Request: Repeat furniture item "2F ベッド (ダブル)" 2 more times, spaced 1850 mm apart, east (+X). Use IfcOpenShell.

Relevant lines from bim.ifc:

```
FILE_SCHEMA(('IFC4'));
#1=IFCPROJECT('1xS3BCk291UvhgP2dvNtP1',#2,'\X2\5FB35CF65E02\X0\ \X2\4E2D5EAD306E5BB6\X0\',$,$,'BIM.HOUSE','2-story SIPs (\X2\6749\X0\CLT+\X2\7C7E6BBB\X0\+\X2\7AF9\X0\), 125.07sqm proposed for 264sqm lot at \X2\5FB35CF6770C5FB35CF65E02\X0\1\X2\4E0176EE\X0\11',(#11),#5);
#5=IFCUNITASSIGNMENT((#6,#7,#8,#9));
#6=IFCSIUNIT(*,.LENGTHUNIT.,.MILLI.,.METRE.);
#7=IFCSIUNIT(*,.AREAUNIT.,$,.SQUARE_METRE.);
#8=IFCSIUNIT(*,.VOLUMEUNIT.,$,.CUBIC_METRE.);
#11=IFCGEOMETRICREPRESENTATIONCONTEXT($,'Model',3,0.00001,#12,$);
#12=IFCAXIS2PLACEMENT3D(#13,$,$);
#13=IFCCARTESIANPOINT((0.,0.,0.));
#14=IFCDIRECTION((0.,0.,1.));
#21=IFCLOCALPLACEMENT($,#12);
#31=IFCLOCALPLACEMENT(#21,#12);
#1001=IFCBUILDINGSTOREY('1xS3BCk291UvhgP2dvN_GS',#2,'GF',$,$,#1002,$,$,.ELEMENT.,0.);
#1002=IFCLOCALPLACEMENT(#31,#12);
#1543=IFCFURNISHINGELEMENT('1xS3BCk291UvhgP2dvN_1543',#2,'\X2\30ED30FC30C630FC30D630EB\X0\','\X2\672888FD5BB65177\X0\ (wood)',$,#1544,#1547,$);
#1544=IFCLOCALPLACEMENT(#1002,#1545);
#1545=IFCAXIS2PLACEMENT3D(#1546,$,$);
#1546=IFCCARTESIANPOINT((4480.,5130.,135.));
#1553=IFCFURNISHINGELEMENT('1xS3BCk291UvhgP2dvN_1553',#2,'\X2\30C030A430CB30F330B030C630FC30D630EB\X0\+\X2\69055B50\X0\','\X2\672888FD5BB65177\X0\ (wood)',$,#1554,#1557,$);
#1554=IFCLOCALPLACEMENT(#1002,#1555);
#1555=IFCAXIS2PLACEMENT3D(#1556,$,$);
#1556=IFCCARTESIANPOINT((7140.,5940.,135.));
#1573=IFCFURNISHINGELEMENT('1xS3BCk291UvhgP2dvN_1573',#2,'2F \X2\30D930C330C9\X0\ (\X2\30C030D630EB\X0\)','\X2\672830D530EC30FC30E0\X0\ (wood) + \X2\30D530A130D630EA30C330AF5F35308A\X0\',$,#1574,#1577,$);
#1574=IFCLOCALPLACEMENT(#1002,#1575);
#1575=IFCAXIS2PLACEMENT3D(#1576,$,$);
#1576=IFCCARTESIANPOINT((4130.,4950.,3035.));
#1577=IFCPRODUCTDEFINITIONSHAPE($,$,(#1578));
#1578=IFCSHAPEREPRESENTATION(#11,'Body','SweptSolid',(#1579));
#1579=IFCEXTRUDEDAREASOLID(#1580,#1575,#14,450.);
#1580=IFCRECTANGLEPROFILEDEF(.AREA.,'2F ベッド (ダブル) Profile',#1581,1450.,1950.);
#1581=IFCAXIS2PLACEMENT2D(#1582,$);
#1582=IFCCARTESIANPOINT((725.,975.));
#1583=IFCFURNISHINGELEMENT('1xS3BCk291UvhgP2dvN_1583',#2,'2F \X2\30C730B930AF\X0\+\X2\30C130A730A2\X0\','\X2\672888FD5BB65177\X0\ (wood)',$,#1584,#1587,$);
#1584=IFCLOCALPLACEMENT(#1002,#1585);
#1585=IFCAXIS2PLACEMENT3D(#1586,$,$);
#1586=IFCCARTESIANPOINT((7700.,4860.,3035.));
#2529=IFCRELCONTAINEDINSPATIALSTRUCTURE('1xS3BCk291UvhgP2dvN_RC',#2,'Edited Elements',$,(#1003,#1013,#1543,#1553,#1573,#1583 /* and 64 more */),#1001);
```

```python
import numpy as np
import ifcopenshell
import ifcopenshell.api.geometry
import ifcopenshell.api.root
import ifcopenshell.util.element
import ifcopenshell.util.placement
import ifcopenshell.util.unit

model = ifcopenshell.open("bim.ifc")
unit_scale = ifcopenshell.util.unit.calculate_unit_scale(model)


def reuse_history(source, copy):
    """copy_class also copies each property set's owner history, people and application; keep the originals."""
    for rel in copy.IsDefinedBy:
        if rel.is_a("IfcRelDefinesByProperties") and (history := rel.RelatingPropertyDefinition.OwnerHistory):
            rel.RelatingPropertyDefinition.OwnerHistory = source.OwnerHistory
            ifcopenshell.util.element.remove_deep2(model, history)


source = model.by_guid("1xS3BCk291UvhgP2dvN_1573")
base = ifcopenshell.util.placement.get_local_placement(source.ObjectPlacement)
step = np.array([1.0, 0.0, 0.0]) * 1.85 / unit_scale

for i in range(1, 3):
    copy = ifcopenshell.api.root.copy_class(model, product=source)
    copy.Representation = ifcopenshell.util.element.copy_deep(
        model, source.Representation, exclude=["IfcGeometricRepresentationContext", "IfcRepresentationMap"]
    )
    reuse_history(source, copy)
    matrix = base.copy()
    matrix[:3, 3] += i * step
    print("added at", matrix[:3, 3].round(3) + 0.0)
    ifcopenshell.api.geometry.edit_object_placement(model, product=copy, matrix=matrix, is_si=False)

model.write("bim_updated.ifc")
```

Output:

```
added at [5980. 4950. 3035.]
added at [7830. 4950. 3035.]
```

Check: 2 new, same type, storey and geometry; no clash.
